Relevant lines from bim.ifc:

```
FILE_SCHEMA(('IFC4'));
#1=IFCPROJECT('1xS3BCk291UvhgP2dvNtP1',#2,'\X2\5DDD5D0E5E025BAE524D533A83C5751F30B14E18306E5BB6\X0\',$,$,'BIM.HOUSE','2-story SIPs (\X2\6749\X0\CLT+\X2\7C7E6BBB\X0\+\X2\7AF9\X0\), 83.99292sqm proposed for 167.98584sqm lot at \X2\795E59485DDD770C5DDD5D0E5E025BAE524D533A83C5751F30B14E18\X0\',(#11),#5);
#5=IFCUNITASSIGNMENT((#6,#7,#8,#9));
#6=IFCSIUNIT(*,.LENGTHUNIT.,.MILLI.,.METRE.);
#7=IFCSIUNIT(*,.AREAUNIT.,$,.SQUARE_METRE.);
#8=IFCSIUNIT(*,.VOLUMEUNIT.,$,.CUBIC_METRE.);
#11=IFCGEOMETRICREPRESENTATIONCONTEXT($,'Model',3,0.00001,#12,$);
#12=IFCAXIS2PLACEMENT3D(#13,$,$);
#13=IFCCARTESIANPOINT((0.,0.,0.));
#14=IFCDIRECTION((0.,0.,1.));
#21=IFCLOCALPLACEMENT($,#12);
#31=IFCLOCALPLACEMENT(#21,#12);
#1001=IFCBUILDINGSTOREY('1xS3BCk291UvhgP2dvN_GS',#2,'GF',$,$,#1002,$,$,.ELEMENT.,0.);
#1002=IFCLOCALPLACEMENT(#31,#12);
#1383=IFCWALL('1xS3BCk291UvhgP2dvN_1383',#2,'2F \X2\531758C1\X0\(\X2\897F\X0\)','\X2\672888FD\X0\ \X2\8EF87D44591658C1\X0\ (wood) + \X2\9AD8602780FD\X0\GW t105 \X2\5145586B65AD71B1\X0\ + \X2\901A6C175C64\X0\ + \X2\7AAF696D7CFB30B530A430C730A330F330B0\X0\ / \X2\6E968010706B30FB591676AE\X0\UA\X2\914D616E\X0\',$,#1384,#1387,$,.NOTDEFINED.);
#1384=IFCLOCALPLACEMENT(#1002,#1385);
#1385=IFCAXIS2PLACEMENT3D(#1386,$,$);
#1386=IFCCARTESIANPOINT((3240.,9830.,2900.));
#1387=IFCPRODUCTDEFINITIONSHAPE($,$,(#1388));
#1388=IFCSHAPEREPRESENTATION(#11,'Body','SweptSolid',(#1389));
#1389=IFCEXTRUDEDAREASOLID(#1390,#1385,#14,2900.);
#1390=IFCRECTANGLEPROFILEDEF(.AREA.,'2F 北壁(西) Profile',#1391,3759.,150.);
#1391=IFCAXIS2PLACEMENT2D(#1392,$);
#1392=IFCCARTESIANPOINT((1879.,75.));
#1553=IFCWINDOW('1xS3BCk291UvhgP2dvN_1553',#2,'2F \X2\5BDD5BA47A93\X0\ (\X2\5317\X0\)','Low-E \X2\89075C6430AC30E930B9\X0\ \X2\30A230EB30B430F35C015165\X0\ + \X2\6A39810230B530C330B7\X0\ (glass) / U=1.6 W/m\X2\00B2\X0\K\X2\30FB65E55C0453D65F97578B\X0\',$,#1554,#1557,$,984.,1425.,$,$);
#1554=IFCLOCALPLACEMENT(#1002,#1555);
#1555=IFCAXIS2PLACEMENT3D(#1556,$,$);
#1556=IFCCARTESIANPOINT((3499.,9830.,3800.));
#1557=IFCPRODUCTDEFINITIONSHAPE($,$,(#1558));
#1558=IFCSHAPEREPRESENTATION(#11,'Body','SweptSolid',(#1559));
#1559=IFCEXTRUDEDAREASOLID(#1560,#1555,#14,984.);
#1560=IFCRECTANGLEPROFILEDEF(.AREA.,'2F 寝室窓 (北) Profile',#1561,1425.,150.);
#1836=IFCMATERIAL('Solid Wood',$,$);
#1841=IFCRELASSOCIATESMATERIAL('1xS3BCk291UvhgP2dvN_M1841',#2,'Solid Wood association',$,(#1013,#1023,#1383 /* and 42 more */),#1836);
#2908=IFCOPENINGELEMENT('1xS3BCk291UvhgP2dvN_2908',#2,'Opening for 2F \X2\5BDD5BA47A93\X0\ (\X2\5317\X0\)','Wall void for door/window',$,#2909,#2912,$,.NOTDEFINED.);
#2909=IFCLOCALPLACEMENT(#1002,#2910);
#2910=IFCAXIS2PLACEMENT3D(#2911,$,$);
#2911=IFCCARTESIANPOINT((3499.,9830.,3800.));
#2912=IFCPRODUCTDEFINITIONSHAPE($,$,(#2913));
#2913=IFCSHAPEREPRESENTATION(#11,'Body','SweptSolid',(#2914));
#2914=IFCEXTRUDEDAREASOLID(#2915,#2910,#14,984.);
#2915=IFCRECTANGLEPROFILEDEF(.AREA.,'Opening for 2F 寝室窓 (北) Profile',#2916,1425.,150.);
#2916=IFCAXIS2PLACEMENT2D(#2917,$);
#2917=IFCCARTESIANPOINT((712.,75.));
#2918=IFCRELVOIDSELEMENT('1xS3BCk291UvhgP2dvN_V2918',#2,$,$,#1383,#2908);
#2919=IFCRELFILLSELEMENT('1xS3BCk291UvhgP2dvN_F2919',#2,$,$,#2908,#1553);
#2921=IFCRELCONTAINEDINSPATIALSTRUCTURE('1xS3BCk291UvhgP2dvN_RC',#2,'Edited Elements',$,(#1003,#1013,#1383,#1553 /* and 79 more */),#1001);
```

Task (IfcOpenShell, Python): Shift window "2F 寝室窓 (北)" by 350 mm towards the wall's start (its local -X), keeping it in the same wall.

```python
import ifcopenshell
import ifcopenshell.api.geometry
import ifcopenshell.util.placement
import ifcopenshell.util.unit

model = ifcopenshell.open("bim.ifc")
unit_scale = ifcopenshell.util.unit.calculate_unit_scale(model)

window = model.by_guid("1xS3BCk291UvhgP2dvN_1553")
opening = window.FillsVoids[0].RelatingOpeningElement
wall = opening.VoidsElements[0].RelatingBuildingElement

wall_matrix = ifcopenshell.util.placement.get_local_placement(wall.ObjectPlacement)
shift = wall_matrix[:3, 0] * -0.35 / unit_scale
before = ifcopenshell.util.placement.get_local_placement(window.ObjectPlacement)[:3, 3].copy()

# The window is not placed relative to its opening, so move both.
for product in (opening, window):
    matrix = ifcopenshell.util.placement.get_local_placement(product.ObjectPlacement)
    matrix[:3, 3] += shift
    ifcopenshell.api.geometry.edit_object_placement(model, product=product, matrix=matrix, is_si=False)

after = ifcopenshell.util.placement.get_local_placement(window.ObjectPlacement)[:3, 3]
print("window moved by", (after - before).round(3) + 0.0)

model.write("bim-out.ifc")
```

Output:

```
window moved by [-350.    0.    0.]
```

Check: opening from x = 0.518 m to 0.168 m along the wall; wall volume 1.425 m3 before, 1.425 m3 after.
